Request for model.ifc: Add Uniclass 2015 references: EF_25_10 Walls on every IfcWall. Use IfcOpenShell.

First a look at what the model holds.

```python
import ifcopenshell

model = ifcopenshell.open("model.ifc")
print(model.schema)
print("classifications:", [c.Name for c in model.by_type("IfcClassification")])
for ifc_class in ("IfcDoor", "IfcRoof", "IfcStair", "IfcWall", "IfcWindow"):
    print(ifc_class, len(model.by_type(ifc_class)))
```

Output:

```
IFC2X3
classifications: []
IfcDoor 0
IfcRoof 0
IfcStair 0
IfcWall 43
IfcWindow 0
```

```python
import ifcopenshell
import ifcopenshell.api.classification

model = ifcopenshell.open("model.ifc")

# IFC2X3 requires Source and Edition and has no link from the project to the system.
system = model.create_entity("IfcClassification", Source="NBS", Edition="2015", Name="Uniclass 2015")

codes = {
    "IfcWall": ("EF_25_10", "Walls"),
}
for ifc_class, (code, name) in codes.items():
    products = model.by_type(ifc_class)
    ifcopenshell.api.classification.add_reference(
        model, products=products, classification=system, identification=code, name=name
    )
    print(code, len(products))

model.write("model_edited.ifc")
```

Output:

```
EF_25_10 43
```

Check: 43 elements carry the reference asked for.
